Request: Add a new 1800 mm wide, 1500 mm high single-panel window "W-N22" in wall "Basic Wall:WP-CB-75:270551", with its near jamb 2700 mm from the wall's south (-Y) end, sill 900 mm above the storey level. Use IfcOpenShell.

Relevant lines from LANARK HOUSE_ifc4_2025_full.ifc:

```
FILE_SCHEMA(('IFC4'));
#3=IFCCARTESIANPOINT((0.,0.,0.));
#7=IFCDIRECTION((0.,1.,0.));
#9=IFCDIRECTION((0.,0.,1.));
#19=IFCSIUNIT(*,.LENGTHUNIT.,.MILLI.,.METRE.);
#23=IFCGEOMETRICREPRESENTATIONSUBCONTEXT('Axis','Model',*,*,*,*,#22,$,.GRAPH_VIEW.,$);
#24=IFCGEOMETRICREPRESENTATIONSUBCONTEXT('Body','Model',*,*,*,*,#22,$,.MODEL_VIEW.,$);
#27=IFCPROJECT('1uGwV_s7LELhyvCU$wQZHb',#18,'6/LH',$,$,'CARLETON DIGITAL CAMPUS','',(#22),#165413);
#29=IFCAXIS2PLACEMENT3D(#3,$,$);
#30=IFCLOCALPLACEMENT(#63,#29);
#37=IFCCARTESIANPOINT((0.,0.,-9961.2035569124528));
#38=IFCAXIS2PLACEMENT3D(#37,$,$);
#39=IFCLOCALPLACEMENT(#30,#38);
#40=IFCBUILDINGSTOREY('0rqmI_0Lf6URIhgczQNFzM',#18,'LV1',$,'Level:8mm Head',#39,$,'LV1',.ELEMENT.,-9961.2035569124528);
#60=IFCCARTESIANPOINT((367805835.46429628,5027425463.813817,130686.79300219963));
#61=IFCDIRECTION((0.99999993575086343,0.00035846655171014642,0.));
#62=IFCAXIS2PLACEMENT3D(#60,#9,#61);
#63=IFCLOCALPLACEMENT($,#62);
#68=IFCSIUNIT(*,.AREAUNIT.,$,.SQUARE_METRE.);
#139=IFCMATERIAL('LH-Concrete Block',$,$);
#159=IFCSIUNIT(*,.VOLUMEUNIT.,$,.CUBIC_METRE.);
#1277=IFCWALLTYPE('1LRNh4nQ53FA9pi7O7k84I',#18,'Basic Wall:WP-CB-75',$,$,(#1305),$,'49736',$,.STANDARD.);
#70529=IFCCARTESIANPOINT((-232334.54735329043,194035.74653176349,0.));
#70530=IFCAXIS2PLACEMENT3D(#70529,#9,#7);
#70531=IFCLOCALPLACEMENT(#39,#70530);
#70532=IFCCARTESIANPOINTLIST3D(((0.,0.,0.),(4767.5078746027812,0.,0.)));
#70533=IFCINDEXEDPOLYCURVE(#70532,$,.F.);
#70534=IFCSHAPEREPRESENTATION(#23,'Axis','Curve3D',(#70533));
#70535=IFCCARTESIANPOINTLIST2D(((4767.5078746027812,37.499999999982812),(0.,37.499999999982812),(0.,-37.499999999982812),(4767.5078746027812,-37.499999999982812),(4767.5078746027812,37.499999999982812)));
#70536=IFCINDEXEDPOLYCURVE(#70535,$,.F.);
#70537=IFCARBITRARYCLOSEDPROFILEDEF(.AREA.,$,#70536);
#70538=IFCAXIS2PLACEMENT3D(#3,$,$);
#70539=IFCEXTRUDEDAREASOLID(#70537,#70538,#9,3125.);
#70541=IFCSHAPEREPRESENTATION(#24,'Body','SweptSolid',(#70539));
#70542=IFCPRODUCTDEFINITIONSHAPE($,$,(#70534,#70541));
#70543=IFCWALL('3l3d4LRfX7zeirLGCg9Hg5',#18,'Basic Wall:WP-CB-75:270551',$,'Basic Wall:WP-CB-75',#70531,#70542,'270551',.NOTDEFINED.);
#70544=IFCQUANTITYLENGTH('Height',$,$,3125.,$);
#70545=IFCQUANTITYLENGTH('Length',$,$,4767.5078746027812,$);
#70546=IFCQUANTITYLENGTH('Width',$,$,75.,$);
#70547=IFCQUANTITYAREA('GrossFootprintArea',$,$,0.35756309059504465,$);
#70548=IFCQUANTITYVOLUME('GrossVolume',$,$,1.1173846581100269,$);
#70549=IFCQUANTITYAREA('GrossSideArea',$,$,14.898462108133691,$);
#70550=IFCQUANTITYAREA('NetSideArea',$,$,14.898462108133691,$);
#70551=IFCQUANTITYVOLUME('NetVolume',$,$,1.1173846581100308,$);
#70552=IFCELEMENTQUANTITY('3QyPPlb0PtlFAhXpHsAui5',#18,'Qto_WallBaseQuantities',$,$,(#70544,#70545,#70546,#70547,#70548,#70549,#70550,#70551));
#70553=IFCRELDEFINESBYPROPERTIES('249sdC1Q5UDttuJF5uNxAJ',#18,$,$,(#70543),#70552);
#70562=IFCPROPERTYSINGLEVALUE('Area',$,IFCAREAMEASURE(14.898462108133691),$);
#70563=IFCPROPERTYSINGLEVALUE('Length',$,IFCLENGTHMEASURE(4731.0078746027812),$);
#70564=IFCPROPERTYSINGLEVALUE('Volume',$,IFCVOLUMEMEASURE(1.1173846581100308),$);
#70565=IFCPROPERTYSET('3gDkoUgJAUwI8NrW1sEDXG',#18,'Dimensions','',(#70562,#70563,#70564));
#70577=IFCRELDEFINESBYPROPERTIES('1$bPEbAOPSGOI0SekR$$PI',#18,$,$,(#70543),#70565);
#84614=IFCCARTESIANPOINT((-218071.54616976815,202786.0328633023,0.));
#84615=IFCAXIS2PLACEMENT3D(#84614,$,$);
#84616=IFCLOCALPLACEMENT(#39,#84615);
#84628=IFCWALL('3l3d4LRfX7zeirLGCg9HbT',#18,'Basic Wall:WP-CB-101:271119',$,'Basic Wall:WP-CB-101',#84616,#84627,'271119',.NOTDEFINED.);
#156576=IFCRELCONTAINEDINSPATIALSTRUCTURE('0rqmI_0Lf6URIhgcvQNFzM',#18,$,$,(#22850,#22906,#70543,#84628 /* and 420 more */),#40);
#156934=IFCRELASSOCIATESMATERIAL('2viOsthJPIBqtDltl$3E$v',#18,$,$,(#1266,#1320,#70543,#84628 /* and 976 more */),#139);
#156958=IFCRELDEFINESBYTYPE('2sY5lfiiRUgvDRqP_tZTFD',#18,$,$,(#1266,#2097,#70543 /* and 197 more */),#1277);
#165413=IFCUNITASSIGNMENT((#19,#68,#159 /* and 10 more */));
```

```python
import numpy as np
import ifcopenshell
import ifcopenshell.api.feature
import ifcopenshell.api.geometry
import ifcopenshell.api.pset
import ifcopenshell.api.root
import ifcopenshell.api.spatial
import ifcopenshell.geom
import ifcopenshell.util.element
import ifcopenshell.util.placement
import ifcopenshell.util.representation
import ifcopenshell.util.shape
import ifcopenshell.util.unit

model = ifcopenshell.open("LANARK HOUSE_ifc4_2025_full.ifc")
unit_scale = ifcopenshell.util.unit.calculate_unit_scale(model)
area_scale = ifcopenshell.util.unit.calculate_unit_scale(model, "AREAUNIT")
volume_scale = ifcopenshell.util.unit.calculate_unit_scale(model, "VOLUMEUNIT")
settings = ifcopenshell.geom.settings()


def volume(element):
    """Net volume in cubic metres, openings subtracted."""
    shape = ifcopenshell.geom.create_shape(settings, element)
    return ifcopenshell.util.shape.get_volume(shape.geometry)


wall = model.by_guid("3l3d4LRfX7zeirLGCg9Hg5")
storey = ifcopenshell.util.element.get_container(wall, ifc_class="IfcBuildingStorey")
context = ifcopenshell.util.representation.get_context(model, "Model", "Body", "MODEL_VIEW")
before = volume(wall)

width, height, from_end, sill = 1.8, 1.5, 2.7, 0.9  # metres

# The wall runs along its own X axis, and the end named is its -X end.
wall_shape = ifcopenshell.geom.create_shape(settings, wall)
x, y, z = ifcopenshell.util.shape.get_vertices(wall_shape.geometry).T
start = x.min() + from_end
face, thickness = float(y.min()), float(y.max() - y.min())
wall_matrix = ifcopenshell.util.placement.get_local_placement(wall.ObjectPlacement)
level = ifcopenshell.util.placement.get_local_placement(storey.ObjectPlacement)[2, 3]


def in_wall(x, y):
    """Placement at x, y metres in the wall's axes, at sill height."""
    matrix = wall_matrix.copy()
    matrix[:, 3] = wall_matrix @ np.array([x / unit_scale, y / unit_scale, 0.0, 1.0])
    matrix[2, 3] = level + sill / unit_scale
    return matrix


# Opening: a box that overshoots both wall faces by 50 mm.
opening = ifcopenshell.api.root.create_entity(model, ifc_class="IfcOpeningElement", predefined_type="OPENING")
box = ifcopenshell.api.geometry.add_wall_representation(
    model, context=context, length=width, height=height, thickness=thickness + 0.1
)
ifcopenshell.api.geometry.assign_representation(model, product=opening, representation=box)
ifcopenshell.api.geometry.edit_object_placement(model, product=opening, matrix=in_wall(start, face - 0.05), is_si=False)
ifcopenshell.api.feature.add_feature(model, feature=opening, element=wall)

window = ifcopenshell.api.root.create_entity(model, ifc_class="IfcWindow", name="W-N22", predefined_type="WINDOW")
window.OverallWidth, window.OverallHeight = width / unit_scale, height / unit_scale
window.PartitioningType = "SINGLE_PANEL"
body = ifcopenshell.api.geometry.add_window_representation(
    model,
    context=context,
    overall_width=window.OverallWidth,
    overall_height=window.OverallHeight,
    partition_type="SINGLE_PANEL",
)
ifcopenshell.api.geometry.assign_representation(model, product=window, representation=body)
ifcopenshell.api.spatial.assign_container(model, products=[window], relating_structure=storey)
ifcopenshell.api.feature.add_filling(model, opening=opening, element=window)

# Centre the window in the wall's thickness.
ifcopenshell.api.geometry.edit_object_placement(model, product=window, matrix=in_wall(start, face), is_si=False)
window_shape = ifcopenshell.geom.create_shape(settings, window)
depth = ifcopenshell.util.shape.get_vertices(window_shape.geometry)[:, 1]
offset = face + thickness / 2 - (depth.min() + depth.max()) / 2
ifcopenshell.api.geometry.edit_object_placement(model, product=window, matrix=in_wall(start, offset), is_si=False)

after = volume(wall)

# Update the wall's stored quantities.
qto = model.by_id(ifcopenshell.util.element.get_pset(wall, "Qto_WallBaseQuantities", should_inherit=False)["id"])
ifcopenshell.api.pset.edit_qto(model, qto=qto, properties={
    "NetSideArea": after / thickness / area_scale,
    "NetVolume": after / volume_scale,
})
pset = model.by_id(ifcopenshell.util.element.get_pset(wall, "Dimensions", should_inherit=False)["id"])
ifcopenshell.api.pset.edit_pset(model, pset=pset, properties={
    "Area": model.create_entity("IfcAreaMeasure", after / thickness / area_scale),
    "Volume": model.create_entity("IfcVolumeMeasure", after / volume_scale),
})

print(f"wall volume {before:.3f} -> {after:.3f} m3")

model.write("LANARK HOUSE_ifc4_2025_full_edited.ifc")
```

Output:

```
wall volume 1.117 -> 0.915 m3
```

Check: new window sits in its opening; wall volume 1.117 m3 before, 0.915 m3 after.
